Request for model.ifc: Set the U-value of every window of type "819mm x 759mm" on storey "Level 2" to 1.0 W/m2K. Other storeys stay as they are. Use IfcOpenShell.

First a look at what the model holds.

```python
import ifcopenshell
import ifcopenshell.util.element

model = ifcopenshell.open("model.ifc")
print(model.schema)
storey = next(s for s in model.by_type("IfcBuildingStorey") if s.Name == "Level 2")
windows = [e for e in ifcopenshell.util.element.get_decomposition(storey) if e.is_a("IfcWindow")]
seen = {}
for e in windows:
    element_type = ifcopenshell.util.element.get_type(e)
    key = (element_type.Name if element_type != e and element_type else None, ifcopenshell.util.element.get_pset(e, "Pset_WindowCommon", "ThermalTransmittance"))
    seen[key] = seen.get(key, 0) + 1
for (name, value), count in sorted(seen.items(), key=str):
    print(count, "x", name, "|", value)
```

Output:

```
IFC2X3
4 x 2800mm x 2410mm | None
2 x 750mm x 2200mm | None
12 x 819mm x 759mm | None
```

```python
import ifcopenshell
import ifcopenshell.api.pset
import ifcopenshell.util.element

model = ifcopenshell.open("model.ifc")

storey = next(s for s in model.by_type("IfcBuildingStorey") if s.Name == "Level 2")
windows = [e for e in ifcopenshell.util.element.get_decomposition(storey) if e.is_a("IfcWindow")]

count = 0
for e in windows:
    element_type = ifcopenshell.util.element.get_type(e)
    if element_type in (None, e) or element_type.Name != "819mm x 759mm":
        continue
    # add_pset returns the element's existing set when there is one.
    pset = ifcopenshell.api.pset.add_pset(model, product=e, name="Pset_WindowCommon")
    ifcopenshell.api.pset.edit_pset(model, pset=pset, properties={"ThermalTransmittance": 1.0})
    count += 1

print(count, "windows updated")

model.write("model_updated.ifc")
```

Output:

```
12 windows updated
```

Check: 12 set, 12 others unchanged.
